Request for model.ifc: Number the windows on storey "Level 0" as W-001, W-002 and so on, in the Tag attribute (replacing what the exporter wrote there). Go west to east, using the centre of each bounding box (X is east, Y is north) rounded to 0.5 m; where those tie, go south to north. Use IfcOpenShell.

First a look at what the model holds.

```python
import ifcopenshell
import ifcopenshell.util.element
import ifcopenshell.util.placement

model = ifcopenshell.open("model.ifc")
print(model.schema)
storey = next(s for s in model.by_type("IfcBuildingStorey") if s.Name == "Level 0")
windows = [e for e in ifcopenshell.util.element.get_decomposition(storey) if e.is_a("IfcWindow")]
for e in sorted(windows, key=lambda e: e.id()):
    origin = ifcopenshell.util.placement.get_local_placement(e.ObjectPlacement)[:3, 3]
    print(e.id(), e.Tag, e.Name, origin.round(2) + 0.0, sep=" | ")
```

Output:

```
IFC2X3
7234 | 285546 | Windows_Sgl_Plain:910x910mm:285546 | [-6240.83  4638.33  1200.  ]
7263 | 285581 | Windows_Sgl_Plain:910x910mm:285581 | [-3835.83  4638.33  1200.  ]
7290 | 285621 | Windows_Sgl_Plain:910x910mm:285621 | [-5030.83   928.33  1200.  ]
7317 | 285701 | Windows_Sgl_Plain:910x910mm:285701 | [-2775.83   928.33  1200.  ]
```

```python
import ifcopenshell
import ifcopenshell.geom
import ifcopenshell.util.element
import ifcopenshell.util.shape

model = ifcopenshell.open("model.ifc")
settings = ifcopenshell.geom.settings()
settings.set("use-world-coords", True)


def centre(element):
    shape = ifcopenshell.geom.create_shape(settings, element)
    return ifcopenshell.util.shape.get_bbox_centroid(shape.geometry)


storey = next(s for s in model.by_type("IfcBuildingStorey") if s.Name == "Level 0")
windows = [e for e in ifcopenshell.util.element.get_decomposition(storey) if e.is_a("IfcWindow")]

# Insertion points can sit at a corner or the storey origin, so sort by the geometry (in metres).
centres = {e: centre(e) for e in windows}
windows.sort(key=lambda e: (round(centres[e][0] / 0.5), centres[e][1]))

for i, e in enumerate(windows, start=1):
    number = f"W-0{i:02d}"
    e.Tag = number
    print(e.id(), number)

model.write("model_edited.ifc")
```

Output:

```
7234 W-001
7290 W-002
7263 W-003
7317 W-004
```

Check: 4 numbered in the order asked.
